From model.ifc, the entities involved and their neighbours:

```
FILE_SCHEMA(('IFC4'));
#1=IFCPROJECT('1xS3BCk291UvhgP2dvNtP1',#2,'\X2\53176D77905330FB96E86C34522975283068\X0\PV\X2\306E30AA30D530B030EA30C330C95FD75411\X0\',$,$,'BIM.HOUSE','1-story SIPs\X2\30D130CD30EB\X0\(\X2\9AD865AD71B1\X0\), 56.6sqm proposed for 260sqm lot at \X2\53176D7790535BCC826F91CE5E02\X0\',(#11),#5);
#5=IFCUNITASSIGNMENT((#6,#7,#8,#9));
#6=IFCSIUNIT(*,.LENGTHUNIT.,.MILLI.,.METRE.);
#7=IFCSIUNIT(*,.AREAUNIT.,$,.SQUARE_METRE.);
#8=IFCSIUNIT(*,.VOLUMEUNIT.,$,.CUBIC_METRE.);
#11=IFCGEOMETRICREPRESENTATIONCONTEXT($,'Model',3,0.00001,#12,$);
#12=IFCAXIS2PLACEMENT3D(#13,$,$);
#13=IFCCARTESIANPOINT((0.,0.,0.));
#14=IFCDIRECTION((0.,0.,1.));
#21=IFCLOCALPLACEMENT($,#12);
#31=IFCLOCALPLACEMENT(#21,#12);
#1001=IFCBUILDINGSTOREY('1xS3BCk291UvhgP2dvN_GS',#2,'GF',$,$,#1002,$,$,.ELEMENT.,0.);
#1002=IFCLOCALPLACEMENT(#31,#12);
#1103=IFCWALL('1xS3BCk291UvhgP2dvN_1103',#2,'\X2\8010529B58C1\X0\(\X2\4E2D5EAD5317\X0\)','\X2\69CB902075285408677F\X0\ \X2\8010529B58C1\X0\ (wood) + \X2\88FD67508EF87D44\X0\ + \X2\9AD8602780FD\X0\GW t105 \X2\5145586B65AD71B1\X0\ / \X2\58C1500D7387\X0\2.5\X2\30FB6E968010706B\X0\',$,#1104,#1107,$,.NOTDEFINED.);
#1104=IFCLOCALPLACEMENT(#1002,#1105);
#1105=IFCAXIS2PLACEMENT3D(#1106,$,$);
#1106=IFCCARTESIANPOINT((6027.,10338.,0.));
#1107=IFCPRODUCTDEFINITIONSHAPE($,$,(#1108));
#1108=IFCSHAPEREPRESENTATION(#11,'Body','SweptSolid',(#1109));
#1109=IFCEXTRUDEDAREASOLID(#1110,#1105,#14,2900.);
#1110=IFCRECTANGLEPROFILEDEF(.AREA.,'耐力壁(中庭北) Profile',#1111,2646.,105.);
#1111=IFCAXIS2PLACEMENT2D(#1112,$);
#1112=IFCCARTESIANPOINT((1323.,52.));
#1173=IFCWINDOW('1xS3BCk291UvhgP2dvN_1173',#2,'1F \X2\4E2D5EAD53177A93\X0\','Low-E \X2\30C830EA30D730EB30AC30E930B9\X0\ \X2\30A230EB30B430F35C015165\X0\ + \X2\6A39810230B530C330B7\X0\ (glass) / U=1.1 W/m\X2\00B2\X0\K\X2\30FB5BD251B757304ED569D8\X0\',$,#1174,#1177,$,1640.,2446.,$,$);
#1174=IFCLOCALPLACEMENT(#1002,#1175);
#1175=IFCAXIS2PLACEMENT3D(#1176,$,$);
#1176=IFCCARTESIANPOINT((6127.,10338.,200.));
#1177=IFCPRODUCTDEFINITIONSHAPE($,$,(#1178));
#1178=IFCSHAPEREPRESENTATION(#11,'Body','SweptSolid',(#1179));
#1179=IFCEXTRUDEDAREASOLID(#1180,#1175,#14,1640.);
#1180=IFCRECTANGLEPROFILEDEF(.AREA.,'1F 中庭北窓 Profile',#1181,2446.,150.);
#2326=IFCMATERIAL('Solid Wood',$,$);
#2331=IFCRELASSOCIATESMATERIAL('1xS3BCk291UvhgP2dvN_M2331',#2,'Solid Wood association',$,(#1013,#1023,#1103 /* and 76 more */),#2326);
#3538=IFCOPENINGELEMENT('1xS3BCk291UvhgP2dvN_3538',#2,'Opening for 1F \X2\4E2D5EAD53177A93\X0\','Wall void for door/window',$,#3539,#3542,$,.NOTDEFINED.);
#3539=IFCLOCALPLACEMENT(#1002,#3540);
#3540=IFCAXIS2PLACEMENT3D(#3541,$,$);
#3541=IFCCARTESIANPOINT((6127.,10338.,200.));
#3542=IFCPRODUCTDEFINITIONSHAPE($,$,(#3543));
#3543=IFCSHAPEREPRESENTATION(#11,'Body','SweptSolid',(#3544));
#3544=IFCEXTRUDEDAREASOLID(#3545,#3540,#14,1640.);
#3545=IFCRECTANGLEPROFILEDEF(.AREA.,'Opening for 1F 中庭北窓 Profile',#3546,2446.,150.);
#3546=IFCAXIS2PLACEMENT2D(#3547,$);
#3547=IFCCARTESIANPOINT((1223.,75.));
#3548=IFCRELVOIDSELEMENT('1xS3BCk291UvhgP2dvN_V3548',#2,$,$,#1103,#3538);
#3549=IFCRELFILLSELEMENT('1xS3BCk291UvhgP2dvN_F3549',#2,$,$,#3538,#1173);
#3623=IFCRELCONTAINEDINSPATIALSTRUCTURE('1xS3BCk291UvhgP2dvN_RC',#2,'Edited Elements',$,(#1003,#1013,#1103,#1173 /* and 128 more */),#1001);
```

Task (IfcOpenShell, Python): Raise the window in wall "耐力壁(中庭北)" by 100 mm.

```python
import numpy as np
import ifcopenshell
import ifcopenshell.api.geometry
import ifcopenshell.util.placement
import ifcopenshell.util.unit

model = ifcopenshell.open("model.ifc")
unit_scale = ifcopenshell.util.unit.calculate_unit_scale(model)

window = model.by_id(1173)
opening = window.FillsVoids[0].RelatingOpeningElement
dz = 100.0

shift = np.array([0.0, 0.0, dz])
# The window is not placed relative to its opening, so move both.
for product in (opening, window):
    matrix = ifcopenshell.util.placement.get_local_placement(product.ObjectPlacement)
    matrix[:3, 3] += shift
    ifcopenshell.api.geometry.edit_object_placement(model, product=product, matrix=matrix, is_si=False)

print(f"moved by {dz * unit_scale:+.3f} m")

model.write("model_rev.ifc")
```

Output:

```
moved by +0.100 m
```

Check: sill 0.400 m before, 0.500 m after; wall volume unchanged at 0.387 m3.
